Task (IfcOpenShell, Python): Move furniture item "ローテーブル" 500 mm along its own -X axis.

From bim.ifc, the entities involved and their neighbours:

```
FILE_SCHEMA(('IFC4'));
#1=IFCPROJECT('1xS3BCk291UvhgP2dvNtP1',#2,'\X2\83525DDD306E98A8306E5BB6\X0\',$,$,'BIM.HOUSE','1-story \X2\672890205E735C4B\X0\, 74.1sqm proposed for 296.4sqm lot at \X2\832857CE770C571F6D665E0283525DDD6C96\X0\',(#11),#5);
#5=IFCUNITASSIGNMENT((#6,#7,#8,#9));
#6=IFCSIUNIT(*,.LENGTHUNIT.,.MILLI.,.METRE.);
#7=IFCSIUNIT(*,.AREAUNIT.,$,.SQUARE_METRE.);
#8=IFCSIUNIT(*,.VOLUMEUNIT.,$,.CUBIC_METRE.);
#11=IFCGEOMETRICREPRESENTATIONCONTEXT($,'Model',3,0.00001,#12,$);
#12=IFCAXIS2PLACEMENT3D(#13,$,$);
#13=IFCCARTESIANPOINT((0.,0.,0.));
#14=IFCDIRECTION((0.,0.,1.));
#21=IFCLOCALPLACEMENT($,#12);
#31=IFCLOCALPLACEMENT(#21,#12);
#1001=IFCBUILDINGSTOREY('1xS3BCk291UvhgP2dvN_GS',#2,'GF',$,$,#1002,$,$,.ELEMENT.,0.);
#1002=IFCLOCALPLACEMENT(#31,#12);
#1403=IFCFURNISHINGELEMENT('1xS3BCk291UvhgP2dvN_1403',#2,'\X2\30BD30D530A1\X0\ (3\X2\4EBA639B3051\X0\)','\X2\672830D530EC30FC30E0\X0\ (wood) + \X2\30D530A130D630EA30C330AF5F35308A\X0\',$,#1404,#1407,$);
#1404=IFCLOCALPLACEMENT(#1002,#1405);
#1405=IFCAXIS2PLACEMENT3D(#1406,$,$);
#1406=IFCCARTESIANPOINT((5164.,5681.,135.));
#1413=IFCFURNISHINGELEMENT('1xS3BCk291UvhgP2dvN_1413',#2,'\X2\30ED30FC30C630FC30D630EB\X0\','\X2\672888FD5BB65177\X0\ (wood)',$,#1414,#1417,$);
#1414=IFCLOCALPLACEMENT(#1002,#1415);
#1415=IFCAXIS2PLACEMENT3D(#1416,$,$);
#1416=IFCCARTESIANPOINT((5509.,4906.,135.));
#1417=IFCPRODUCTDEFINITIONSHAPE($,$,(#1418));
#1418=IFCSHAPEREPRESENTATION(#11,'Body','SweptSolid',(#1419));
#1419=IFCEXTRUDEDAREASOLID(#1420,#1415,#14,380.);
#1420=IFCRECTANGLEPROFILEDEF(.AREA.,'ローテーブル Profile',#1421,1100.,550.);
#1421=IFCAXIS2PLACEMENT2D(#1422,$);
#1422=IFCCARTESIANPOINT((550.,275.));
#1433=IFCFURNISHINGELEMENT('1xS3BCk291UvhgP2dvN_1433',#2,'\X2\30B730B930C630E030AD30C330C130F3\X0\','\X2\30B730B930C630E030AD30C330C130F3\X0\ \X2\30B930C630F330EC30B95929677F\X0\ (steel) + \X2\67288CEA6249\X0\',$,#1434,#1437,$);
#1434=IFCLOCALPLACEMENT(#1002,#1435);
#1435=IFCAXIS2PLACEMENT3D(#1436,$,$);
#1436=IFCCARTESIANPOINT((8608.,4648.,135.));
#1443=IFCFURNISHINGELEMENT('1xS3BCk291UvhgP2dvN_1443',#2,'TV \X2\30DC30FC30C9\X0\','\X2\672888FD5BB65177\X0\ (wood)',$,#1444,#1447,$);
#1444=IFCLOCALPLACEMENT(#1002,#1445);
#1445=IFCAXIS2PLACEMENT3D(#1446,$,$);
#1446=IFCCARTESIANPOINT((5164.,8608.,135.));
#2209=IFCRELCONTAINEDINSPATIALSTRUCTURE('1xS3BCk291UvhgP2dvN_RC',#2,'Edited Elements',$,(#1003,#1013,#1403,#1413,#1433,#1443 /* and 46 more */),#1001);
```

```python
import ifcopenshell
import ifcopenshell.api.geometry
import ifcopenshell.util.placement
import ifcopenshell.util.unit

model = ifcopenshell.open("bim.ifc")
unit_scale = ifcopenshell.util.unit.calculate_unit_scale(model)

item = model.by_id(1413)
matrix = ifcopenshell.util.placement.get_local_placement(item.ObjectPlacement)
matrix[:3, 3] -= matrix[:3, 0] * 0.5 / unit_scale
ifcopenshell.api.geometry.edit_object_placement(model, product=item, matrix=matrix, is_si=False)

print(ifcopenshell.util.placement.get_local_placement(item.ObjectPlacement).round(3) + 0.0)

model.write("bim_edited.ifc")
```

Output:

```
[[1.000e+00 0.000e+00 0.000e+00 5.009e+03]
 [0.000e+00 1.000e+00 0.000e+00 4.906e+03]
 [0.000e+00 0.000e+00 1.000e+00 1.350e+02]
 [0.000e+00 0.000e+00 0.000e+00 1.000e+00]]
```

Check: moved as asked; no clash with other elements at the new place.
